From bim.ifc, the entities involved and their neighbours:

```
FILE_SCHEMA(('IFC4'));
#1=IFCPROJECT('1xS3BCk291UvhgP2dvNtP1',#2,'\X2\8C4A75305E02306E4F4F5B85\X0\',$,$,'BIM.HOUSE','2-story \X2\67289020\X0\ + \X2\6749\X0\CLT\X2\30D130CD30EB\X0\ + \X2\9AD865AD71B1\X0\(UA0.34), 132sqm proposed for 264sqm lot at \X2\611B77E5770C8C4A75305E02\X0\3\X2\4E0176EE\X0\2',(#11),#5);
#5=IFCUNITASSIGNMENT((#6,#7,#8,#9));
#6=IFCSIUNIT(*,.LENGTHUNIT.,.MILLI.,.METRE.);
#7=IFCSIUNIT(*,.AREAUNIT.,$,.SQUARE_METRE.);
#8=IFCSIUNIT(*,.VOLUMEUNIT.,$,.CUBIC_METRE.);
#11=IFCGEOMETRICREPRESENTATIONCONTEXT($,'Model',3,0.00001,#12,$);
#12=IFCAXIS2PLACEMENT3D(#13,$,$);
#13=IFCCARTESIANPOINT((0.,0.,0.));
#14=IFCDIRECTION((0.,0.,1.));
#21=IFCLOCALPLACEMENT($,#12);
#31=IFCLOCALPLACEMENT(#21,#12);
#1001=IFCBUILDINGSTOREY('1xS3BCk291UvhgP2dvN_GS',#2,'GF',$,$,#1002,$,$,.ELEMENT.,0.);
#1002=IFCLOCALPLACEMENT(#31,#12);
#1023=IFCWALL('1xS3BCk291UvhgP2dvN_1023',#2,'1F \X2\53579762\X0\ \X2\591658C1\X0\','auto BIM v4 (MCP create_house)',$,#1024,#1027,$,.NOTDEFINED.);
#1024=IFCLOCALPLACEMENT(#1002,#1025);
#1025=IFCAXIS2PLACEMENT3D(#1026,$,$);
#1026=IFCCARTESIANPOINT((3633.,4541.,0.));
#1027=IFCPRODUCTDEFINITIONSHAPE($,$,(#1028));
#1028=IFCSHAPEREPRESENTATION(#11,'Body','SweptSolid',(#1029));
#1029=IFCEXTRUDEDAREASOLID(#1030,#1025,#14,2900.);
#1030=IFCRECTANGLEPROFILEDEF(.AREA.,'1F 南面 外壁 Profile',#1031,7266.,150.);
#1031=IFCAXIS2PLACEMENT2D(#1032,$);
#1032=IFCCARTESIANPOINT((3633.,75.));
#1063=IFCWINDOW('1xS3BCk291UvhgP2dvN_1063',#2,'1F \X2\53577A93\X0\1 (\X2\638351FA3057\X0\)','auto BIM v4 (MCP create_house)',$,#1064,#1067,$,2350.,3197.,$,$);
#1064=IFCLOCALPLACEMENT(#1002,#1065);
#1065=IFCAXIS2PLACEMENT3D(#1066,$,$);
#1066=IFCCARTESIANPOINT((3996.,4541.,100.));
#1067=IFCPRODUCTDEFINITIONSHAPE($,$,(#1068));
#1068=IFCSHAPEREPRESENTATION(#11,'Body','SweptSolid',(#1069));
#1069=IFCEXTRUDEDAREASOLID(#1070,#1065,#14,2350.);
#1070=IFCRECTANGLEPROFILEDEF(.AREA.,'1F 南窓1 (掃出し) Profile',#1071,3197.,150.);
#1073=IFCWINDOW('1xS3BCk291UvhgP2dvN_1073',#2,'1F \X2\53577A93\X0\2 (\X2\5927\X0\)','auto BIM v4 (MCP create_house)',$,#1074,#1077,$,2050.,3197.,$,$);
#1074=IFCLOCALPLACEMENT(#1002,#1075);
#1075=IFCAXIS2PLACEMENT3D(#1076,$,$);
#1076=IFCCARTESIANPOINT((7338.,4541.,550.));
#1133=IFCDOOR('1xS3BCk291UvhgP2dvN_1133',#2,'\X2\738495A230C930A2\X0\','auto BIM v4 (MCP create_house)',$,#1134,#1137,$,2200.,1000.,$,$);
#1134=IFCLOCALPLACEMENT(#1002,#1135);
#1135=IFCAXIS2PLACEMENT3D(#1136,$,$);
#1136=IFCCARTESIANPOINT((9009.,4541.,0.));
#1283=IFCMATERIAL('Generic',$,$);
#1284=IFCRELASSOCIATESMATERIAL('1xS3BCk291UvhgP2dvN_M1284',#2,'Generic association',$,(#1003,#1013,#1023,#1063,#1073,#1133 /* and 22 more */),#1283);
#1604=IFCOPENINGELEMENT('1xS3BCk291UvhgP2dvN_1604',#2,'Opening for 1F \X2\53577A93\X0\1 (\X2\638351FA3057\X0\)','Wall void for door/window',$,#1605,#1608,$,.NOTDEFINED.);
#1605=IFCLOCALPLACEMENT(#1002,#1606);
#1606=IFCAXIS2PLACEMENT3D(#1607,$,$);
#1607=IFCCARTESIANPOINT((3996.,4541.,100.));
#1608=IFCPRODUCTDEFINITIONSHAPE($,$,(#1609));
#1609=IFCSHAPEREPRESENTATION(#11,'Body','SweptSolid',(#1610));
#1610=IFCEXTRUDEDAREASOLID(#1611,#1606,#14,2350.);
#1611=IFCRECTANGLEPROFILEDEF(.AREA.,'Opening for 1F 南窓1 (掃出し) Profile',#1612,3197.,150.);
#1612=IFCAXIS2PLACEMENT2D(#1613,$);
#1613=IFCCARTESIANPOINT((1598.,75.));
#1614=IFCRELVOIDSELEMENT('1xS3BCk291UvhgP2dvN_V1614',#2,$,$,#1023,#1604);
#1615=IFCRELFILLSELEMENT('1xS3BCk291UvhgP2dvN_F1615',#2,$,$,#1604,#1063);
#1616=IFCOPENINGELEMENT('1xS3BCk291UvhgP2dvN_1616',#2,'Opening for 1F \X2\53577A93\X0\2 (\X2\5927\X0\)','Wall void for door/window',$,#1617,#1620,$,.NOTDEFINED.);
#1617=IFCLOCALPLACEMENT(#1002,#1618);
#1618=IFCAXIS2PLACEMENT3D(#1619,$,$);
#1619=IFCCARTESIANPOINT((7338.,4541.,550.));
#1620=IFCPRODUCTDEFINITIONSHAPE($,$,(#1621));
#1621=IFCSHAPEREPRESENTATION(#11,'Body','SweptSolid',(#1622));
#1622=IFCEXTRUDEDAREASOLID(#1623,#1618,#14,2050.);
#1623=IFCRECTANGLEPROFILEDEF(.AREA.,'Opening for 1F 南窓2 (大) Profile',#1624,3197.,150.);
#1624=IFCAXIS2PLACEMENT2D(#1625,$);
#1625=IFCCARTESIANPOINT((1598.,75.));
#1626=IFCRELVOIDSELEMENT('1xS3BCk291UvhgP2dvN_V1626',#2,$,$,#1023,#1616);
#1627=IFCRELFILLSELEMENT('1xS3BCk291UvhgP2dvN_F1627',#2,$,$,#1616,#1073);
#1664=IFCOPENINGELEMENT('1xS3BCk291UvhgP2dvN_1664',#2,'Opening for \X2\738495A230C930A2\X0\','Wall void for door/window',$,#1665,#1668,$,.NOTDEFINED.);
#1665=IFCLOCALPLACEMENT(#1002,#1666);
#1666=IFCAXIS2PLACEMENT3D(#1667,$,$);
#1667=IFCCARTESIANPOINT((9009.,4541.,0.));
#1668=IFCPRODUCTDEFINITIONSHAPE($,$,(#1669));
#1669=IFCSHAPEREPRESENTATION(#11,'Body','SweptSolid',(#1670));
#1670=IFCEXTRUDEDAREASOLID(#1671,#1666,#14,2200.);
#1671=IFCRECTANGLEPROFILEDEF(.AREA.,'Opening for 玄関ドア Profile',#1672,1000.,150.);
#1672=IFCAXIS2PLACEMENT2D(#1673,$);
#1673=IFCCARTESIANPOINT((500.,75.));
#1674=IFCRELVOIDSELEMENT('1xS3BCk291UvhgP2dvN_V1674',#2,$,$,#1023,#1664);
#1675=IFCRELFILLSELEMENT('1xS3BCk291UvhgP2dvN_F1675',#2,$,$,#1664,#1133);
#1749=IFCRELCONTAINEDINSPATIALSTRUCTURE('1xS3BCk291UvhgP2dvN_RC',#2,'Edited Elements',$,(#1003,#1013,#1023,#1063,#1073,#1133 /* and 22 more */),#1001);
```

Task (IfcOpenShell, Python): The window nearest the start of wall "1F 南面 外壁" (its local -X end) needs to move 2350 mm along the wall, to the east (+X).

```python
import ifcopenshell
import ifcopenshell.api.geometry
import ifcopenshell.util.placement

model = ifcopenshell.open("bim.ifc")

window = model.by_guid("1xS3BCk291UvhgP2dvN_1063")
opening = window.FillsVoids[0].RelatingOpeningElement
wall = opening.VoidsElements[0].RelatingBuildingElement

wall_matrix = ifcopenshell.util.placement.get_local_placement(wall.ObjectPlacement)
shift = wall_matrix[:3, 0] * 2350.0
before = ifcopenshell.util.placement.get_local_placement(window.ObjectPlacement)[:3, 3].copy()

# The window is not placed relative to its opening, so move both.
for product in (opening, window):
    matrix = ifcopenshell.util.placement.get_local_placement(product.ObjectPlacement)
    matrix[:3, 3] += shift
    ifcopenshell.api.geometry.edit_object_placement(model, product=product, matrix=matrix, is_si=False)

after = ifcopenshell.util.placement.get_local_placement(window.ObjectPlacement)[:3, 3]
print("window moved by", (after - before).round(3) + 0.0)

model.write("bim-out.ifc")
```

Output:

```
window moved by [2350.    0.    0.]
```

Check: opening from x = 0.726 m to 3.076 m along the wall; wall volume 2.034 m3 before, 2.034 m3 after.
